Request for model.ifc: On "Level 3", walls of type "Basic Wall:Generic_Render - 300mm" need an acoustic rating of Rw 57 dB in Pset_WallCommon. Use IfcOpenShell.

First a look at what the model holds.

```python
import ifcopenshell
import ifcopenshell.util.element

model = ifcopenshell.open("model.ifc")
print(model.schema)
storey = next(s for s in model.by_type("IfcBuildingStorey") if s.Name == "Level 3")
walls = [e for e in ifcopenshell.util.element.get_decomposition(storey) if e.is_a("IfcWall")]
seen = {}
for e in walls:
    element_type = ifcopenshell.util.element.get_type(e)
    key = (element_type.Name if element_type != e and element_type else None, ifcopenshell.util.element.get_pset(e, "Pset_WallCommon", "AcousticRating"))
    seen[key] = seen.get(key, 0) + 1
for (name, value), count in sorted(seen.items(), key=str):
    print(count, "x", name, "|", value)
```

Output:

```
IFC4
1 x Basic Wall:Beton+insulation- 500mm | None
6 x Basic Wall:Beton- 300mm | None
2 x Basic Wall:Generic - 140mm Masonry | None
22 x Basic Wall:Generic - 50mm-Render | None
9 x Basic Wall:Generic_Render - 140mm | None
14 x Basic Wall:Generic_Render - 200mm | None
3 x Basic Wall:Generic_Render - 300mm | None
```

```python
import ifcopenshell
import ifcopenshell.api.pset
import ifcopenshell.util.element

model = ifcopenshell.open("model.ifc")

storey = next(s for s in model.by_type("IfcBuildingStorey") if s.Name == "Level 3")
walls = [e for e in ifcopenshell.util.element.get_decomposition(storey) if e.is_a("IfcWall")]

count = 0
for e in walls:
    element_type = ifcopenshell.util.element.get_type(e)
    if element_type in (None, e) or element_type.Name != "Basic Wall:Generic_Render - 300mm":
        continue
    # add_pset returns the element's existing set when there is one.
    pset = ifcopenshell.api.pset.add_pset(model, product=e, name="Pset_WallCommon")
    ifcopenshell.api.pset.edit_pset(model, pset=pset, properties={"AcousticRating": "Rw 57 dB"})
    count += 1

print(count, "walls updated")

model.write("model_v2.ifc")
```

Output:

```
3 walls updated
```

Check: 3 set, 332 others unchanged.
